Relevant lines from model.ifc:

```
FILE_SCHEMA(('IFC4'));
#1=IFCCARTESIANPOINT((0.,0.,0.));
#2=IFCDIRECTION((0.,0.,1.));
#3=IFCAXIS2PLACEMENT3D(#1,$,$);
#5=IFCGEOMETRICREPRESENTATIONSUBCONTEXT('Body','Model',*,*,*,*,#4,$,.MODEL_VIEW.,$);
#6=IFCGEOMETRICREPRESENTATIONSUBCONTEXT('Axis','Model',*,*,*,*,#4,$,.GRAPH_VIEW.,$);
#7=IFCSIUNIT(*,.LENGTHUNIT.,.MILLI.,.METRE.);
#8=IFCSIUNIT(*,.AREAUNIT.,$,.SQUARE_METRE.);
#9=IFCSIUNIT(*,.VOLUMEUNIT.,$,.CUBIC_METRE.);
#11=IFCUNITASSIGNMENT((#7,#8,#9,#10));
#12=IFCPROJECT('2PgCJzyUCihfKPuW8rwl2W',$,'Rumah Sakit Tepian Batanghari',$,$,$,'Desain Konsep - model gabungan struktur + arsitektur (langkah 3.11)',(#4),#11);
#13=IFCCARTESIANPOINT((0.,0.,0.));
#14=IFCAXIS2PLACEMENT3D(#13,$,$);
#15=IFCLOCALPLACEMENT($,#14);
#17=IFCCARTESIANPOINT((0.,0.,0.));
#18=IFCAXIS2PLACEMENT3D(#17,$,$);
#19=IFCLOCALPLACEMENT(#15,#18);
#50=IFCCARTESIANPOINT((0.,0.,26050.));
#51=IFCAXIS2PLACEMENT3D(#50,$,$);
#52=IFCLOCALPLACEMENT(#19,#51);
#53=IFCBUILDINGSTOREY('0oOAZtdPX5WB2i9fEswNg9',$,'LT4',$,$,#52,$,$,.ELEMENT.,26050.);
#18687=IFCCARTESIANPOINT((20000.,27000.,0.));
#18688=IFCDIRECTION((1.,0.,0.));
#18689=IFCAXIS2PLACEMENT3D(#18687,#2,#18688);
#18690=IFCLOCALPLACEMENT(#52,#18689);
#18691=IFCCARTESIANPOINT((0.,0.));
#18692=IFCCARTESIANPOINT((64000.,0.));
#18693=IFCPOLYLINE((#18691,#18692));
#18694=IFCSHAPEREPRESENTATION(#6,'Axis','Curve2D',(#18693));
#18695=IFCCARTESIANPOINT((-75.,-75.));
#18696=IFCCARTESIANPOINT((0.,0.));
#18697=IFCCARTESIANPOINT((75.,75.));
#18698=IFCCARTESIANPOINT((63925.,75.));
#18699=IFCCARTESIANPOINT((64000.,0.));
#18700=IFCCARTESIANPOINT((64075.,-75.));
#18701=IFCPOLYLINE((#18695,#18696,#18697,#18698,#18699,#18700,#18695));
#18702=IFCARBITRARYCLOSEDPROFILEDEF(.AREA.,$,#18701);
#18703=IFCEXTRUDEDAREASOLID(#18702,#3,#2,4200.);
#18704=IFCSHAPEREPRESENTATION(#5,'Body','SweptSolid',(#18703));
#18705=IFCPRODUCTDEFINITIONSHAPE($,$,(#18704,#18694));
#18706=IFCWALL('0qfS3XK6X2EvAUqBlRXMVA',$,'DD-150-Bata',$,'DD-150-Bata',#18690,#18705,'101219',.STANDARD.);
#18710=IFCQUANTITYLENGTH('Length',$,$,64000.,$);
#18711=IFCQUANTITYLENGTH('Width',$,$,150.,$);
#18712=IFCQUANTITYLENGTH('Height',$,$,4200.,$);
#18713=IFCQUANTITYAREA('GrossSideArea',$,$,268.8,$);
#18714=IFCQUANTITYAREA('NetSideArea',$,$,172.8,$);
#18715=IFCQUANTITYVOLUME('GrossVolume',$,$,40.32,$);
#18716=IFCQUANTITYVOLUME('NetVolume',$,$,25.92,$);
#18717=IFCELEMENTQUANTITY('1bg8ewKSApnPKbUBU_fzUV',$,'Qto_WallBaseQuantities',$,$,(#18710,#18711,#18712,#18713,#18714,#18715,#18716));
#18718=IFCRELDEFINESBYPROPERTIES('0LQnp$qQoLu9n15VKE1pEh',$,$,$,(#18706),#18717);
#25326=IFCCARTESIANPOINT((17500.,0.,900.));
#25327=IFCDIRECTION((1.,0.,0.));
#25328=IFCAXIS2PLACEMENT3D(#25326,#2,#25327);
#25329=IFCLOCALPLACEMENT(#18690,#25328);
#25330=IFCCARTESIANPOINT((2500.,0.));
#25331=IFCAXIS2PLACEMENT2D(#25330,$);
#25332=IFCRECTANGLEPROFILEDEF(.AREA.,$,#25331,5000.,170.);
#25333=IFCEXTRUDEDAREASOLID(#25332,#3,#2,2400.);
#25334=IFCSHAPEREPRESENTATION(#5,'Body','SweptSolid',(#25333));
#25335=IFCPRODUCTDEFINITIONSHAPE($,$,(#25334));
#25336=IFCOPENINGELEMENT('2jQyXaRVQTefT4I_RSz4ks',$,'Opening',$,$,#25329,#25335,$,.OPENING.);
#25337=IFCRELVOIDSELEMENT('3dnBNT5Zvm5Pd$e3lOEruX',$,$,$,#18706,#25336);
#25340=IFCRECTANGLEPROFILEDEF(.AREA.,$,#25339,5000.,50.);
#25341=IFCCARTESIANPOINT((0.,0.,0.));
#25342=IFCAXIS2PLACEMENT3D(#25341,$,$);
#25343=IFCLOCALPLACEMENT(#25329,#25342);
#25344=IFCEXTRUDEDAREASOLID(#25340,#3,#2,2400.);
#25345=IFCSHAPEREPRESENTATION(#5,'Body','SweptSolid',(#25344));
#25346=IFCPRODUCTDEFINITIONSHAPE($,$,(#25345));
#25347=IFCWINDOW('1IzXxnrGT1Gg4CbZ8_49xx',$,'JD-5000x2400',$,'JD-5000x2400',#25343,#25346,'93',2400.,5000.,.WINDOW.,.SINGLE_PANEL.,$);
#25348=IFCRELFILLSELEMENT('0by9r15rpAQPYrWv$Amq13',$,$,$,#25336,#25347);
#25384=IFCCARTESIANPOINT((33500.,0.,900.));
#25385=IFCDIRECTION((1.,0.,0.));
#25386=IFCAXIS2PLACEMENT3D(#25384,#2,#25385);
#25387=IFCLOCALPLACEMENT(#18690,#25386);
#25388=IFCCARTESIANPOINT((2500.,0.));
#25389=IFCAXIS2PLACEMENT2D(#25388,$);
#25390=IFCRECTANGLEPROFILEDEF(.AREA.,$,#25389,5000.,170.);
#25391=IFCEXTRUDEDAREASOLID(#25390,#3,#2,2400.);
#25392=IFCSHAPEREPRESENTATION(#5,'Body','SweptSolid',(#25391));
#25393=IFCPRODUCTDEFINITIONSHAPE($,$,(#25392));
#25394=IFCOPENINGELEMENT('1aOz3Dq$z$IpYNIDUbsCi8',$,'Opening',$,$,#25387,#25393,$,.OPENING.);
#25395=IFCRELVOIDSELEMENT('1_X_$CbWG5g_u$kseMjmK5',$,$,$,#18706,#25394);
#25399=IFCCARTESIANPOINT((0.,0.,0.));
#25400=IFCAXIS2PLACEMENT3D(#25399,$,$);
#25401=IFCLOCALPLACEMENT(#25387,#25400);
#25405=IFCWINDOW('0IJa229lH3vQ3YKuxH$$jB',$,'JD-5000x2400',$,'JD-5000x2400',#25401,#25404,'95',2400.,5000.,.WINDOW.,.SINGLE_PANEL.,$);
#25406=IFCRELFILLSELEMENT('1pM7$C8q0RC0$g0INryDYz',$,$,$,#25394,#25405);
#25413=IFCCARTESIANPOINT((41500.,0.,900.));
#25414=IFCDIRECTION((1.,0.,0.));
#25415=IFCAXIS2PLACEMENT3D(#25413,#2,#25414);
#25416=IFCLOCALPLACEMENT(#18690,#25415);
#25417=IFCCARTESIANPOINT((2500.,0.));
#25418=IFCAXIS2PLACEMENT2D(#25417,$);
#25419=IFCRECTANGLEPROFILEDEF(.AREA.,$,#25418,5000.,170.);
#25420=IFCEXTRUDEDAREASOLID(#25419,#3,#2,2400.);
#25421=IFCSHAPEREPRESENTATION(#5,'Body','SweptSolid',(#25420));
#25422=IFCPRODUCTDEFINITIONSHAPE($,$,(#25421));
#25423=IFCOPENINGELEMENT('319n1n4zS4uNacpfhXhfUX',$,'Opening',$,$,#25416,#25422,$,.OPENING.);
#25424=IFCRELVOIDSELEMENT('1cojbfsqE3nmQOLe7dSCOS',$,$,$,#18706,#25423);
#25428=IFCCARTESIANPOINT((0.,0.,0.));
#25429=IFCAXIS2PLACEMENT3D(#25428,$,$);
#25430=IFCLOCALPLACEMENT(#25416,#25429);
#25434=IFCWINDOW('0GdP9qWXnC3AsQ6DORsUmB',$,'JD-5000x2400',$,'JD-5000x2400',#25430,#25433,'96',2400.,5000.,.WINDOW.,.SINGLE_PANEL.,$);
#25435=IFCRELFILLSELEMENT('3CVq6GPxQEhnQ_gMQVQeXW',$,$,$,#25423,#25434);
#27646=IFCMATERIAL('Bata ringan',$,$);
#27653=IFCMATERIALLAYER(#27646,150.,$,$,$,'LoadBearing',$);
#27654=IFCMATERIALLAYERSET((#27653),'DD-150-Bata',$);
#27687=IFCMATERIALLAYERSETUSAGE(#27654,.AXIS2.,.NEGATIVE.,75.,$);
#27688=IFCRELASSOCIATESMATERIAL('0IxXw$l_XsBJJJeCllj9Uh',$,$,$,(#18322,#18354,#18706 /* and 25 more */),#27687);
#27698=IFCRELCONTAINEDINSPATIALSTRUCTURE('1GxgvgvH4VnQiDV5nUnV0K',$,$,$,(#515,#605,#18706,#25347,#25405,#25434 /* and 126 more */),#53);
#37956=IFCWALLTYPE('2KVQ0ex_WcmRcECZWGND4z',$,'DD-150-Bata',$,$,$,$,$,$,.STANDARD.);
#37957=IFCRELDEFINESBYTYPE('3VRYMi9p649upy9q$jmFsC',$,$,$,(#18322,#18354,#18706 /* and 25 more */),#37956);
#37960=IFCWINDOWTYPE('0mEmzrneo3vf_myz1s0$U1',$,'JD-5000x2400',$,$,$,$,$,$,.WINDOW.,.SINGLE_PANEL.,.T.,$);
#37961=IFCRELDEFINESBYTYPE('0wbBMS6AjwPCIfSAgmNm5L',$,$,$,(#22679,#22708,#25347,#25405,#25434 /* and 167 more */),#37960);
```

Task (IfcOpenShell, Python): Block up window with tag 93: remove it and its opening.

```python
import ifcopenshell
import ifcopenshell.api.feature
import ifcopenshell.api.pset
import ifcopenshell.api.root
import ifcopenshell.geom
import ifcopenshell.util.element
import ifcopenshell.util.shape
import ifcopenshell.util.unit

model = ifcopenshell.open("model.ifc")
area_scale = ifcopenshell.util.unit.calculate_unit_scale(model, "AREAUNIT")
volume_scale = ifcopenshell.util.unit.calculate_unit_scale(model, "VOLUMEUNIT")
settings = ifcopenshell.geom.settings()


def volume(element):
    """Net volume in cubic metres, openings subtracted."""
    shape = ifcopenshell.geom.create_shape(settings, element)
    return ifcopenshell.util.shape.get_volume(shape.geometry)


window = model.by_guid("1IzXxnrGT1Gg4CbZ8_49xx")
opening = window.FillsVoids[0].RelatingOpeningElement
wall = opening.VoidsElements[0].RelatingBuildingElement
before = volume(wall)

ifcopenshell.api.root.remove_product(model, product=window)
ifcopenshell.api.feature.remove_feature(model, feature=opening)

after = volume(wall)
thickness = 0.15  # wall thickness in metres

# Update the wall's stored quantities.
qto = model.by_id(ifcopenshell.util.element.get_pset(wall, "Qto_WallBaseQuantities", should_inherit=False)["id"])
ifcopenshell.api.pset.edit_qto(model, qto=qto, properties={
    "NetSideArea": after / thickness / area_scale,
    "NetVolume": after / volume_scale,
})

print(f"wall volume {before:.3f} -> {after:.3f} m3")

model.write("model_rev.ifc")
```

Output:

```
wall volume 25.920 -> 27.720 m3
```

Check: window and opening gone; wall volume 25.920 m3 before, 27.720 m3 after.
